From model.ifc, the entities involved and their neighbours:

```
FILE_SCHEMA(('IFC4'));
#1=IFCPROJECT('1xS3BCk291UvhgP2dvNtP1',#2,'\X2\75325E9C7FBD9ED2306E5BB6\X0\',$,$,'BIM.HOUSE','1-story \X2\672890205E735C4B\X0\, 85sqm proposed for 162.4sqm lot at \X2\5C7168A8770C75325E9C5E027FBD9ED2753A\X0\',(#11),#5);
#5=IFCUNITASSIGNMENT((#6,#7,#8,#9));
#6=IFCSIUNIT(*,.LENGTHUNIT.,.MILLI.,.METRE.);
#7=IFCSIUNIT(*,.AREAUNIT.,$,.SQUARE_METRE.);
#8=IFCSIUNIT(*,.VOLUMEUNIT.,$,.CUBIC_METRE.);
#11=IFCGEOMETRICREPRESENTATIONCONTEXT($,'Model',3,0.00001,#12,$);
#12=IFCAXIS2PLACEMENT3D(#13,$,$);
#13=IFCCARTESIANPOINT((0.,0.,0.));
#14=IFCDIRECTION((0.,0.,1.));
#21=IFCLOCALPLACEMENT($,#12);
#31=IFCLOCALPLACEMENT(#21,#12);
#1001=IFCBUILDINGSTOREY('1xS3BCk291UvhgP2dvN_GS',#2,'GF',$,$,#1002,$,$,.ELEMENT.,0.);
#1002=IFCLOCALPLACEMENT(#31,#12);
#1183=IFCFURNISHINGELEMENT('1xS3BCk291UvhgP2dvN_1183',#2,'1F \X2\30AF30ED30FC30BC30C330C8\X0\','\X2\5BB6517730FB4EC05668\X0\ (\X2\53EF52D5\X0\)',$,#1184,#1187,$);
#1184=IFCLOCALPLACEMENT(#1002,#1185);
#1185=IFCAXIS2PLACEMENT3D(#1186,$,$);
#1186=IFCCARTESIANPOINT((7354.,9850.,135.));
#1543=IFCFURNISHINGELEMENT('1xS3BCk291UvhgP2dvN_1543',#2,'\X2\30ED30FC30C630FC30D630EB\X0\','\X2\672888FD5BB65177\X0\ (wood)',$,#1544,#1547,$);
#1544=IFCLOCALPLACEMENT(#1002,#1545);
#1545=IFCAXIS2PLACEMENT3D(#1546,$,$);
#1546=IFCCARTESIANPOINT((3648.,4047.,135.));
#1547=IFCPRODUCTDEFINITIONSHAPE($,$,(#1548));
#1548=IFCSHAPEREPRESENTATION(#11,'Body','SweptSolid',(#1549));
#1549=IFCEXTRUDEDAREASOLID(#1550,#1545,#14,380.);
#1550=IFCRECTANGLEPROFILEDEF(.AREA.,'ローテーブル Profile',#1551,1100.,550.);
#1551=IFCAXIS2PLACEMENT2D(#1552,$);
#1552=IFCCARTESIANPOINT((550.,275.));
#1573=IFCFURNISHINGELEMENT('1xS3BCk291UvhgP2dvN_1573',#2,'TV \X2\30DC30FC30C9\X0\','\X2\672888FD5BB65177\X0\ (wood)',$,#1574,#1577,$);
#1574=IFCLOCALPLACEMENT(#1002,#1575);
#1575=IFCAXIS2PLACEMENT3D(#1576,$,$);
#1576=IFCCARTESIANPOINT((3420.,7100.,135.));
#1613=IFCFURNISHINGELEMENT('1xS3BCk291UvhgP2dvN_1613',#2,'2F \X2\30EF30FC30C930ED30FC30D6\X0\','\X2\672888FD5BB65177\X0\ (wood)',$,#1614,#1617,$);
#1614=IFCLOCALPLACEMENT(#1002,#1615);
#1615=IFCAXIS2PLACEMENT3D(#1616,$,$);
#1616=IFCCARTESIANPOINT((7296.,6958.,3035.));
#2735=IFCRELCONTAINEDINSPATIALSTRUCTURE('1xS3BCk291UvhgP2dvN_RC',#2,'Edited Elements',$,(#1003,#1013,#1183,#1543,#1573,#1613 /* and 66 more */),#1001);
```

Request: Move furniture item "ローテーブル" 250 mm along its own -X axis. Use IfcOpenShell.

```python
import ifcopenshell
import ifcopenshell.api.geometry
import ifcopenshell.util.placement

model = ifcopenshell.open("model.ifc")

item = model.by_guid("1xS3BCk291UvhgP2dvN_1543")
matrix = ifcopenshell.util.placement.get_local_placement(item.ObjectPlacement)
matrix[:3, 3] -= matrix[:3, 0] * 250.0
ifcopenshell.api.geometry.edit_object_placement(model, product=item, matrix=matrix, is_si=False)

print(ifcopenshell.util.placement.get_local_placement(item.ObjectPlacement).round(3) + 0.0)

model.write("model_edited.ifc")
```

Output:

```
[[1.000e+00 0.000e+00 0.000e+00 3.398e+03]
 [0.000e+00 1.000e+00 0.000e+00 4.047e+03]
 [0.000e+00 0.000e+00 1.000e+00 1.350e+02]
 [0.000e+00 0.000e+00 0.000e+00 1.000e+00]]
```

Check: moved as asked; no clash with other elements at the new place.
